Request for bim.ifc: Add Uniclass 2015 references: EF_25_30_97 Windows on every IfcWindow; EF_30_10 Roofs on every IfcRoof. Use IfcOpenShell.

First a look at what the model holds.

```python
import ifcopenshell

model = ifcopenshell.open("bim.ifc")
print(model.schema)
print("classifications:", [c.Name for c in model.by_type("IfcClassification")])
for ifc_class in ("IfcDoor", "IfcRoof", "IfcStair", "IfcWall", "IfcWindow"):
    print(ifc_class, len(model.by_type(ifc_class)))
```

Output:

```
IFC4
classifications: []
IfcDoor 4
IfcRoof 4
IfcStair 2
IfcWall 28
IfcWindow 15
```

```python
import ifcopenshell
import ifcopenshell.api.classification

model = ifcopenshell.open("bim.ifc")

system = ifcopenshell.api.classification.add_classification(model, classification="Uniclass 2015")

codes = {
    "IfcWindow": ("EF_25_30_97", "Windows"),
    "IfcRoof": ("EF_30_10", "Roofs"),
}
for ifc_class, (code, name) in codes.items():
    products = model.by_type(ifc_class)
    ifcopenshell.api.classification.add_reference(
        model, products=products, classification=system, identification=code, name=name
    )
    print(code, len(products))

model.write("bim_updated.ifc")
```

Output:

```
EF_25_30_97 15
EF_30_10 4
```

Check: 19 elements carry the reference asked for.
